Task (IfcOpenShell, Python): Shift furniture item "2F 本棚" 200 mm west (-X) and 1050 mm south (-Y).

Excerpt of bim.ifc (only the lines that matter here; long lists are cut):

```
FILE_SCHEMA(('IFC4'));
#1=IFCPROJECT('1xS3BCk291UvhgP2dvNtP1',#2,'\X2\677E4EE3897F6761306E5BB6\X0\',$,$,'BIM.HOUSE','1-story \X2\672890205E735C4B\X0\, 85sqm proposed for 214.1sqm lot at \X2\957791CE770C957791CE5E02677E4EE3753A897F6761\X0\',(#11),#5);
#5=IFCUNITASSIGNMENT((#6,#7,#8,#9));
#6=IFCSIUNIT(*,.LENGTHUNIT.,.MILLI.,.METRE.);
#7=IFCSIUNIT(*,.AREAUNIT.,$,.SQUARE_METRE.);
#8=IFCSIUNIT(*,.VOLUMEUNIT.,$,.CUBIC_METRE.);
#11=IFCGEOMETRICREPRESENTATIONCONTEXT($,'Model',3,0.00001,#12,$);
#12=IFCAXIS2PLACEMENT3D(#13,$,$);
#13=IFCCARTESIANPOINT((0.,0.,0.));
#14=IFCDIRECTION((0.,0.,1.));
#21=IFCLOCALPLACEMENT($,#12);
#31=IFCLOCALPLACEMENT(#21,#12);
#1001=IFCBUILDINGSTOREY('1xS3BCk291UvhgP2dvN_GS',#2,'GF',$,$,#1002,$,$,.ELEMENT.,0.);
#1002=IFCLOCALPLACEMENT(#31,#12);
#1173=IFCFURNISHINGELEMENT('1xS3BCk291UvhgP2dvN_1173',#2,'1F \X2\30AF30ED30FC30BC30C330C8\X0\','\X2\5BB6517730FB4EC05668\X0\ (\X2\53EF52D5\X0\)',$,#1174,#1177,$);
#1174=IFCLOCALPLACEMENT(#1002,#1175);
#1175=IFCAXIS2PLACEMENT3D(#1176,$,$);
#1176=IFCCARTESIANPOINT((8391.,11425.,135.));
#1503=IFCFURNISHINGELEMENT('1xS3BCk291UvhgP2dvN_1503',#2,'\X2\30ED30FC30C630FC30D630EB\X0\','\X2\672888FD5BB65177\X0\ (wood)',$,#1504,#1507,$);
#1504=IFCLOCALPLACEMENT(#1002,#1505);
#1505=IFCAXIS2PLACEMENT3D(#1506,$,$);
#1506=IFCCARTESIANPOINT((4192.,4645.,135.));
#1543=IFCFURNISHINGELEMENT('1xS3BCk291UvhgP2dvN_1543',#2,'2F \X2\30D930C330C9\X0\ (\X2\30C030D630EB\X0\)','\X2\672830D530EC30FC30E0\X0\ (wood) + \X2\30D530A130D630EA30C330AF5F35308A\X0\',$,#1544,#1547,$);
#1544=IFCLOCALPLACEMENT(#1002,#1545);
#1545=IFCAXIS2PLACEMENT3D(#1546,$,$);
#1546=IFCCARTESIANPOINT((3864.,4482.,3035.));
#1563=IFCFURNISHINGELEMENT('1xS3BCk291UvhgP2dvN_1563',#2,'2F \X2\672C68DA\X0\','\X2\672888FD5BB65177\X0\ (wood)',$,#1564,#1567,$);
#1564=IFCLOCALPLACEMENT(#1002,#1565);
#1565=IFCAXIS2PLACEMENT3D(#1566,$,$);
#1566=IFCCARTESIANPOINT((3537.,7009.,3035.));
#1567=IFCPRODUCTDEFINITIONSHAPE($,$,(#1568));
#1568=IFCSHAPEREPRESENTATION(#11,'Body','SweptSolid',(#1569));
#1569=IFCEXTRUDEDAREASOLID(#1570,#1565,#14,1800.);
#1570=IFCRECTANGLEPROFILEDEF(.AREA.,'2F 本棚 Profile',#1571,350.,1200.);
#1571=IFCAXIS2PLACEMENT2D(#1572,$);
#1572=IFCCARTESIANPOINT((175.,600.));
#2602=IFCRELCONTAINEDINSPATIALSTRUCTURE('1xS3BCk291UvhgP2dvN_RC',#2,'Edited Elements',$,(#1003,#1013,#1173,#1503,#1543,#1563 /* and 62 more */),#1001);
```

```python
import ifcopenshell
import ifcopenshell.api.geometry
import ifcopenshell.util.placement
import ifcopenshell.util.unit

model = ifcopenshell.open("bim.ifc")
unit_scale = ifcopenshell.util.unit.calculate_unit_scale(model)

item = model.by_guid("1xS3BCk291UvhgP2dvN_1563")
matrix = ifcopenshell.util.placement.get_local_placement(item.ObjectPlacement)
matrix[0, 3] -= 0.2 / unit_scale
matrix[1, 3] -= 1.05 / unit_scale
ifcopenshell.api.geometry.edit_object_placement(model, product=item, matrix=matrix, is_si=False)

print(ifcopenshell.util.placement.get_local_placement(item.ObjectPlacement).round(3) + 0.0)

model.write("bim_updated.ifc")
```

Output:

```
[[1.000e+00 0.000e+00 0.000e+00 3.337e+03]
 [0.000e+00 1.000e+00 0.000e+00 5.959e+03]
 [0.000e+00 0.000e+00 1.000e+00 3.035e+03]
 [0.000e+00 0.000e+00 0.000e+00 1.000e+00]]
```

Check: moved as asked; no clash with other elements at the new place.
